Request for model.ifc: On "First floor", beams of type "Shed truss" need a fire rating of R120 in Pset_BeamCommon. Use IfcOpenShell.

First a look at what the model holds.

```python
import ifcopenshell
import ifcopenshell.util.element

model = ifcopenshell.open("model.ifc")
print(model.schema)
storey = next(s for s in model.by_type("IfcBuildingStorey") if s.Name == "First floor")
beams = [e for e in ifcopenshell.util.element.get_decomposition(storey) if e.is_a("IfcBeam")]
seen = {}
for e in beams:
    element_type = ifcopenshell.util.element.get_type(e)
    key = (element_type.Name if element_type != e and element_type else None, ifcopenshell.util.element.get_pset(e, "Pset_BeamCommon", "FireRating"))
    seen[key] = seen.get(key, 0) + 1
for (name, value), count in sorted(seen.items(), key=str):
    print(count, "x", name, "|", value)
```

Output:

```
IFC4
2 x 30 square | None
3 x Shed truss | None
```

```python
import ifcopenshell
import ifcopenshell.api.pset
import ifcopenshell.util.element

model = ifcopenshell.open("model.ifc")

storey = next(s for s in model.by_type("IfcBuildingStorey") if s.Name == "First floor")
beams = [e for e in ifcopenshell.util.element.get_decomposition(storey) if e.is_a("IfcBeam")]

count = 0
for e in beams:
    element_type = ifcopenshell.util.element.get_type(e)
    if element_type in (None, e) or element_type.Name != "Shed truss":
        continue
    # add_pset returns the element's existing set when there is one.
    pset = ifcopenshell.api.pset.add_pset(model, product=e, name="Pset_BeamCommon")
    ifcopenshell.api.pset.edit_pset(model, pset=pset, properties={"FireRating": "R120"})
    count += 1

print(count, "beams updated")

model.write("model_updated.ifc")
```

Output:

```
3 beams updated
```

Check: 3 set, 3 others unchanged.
